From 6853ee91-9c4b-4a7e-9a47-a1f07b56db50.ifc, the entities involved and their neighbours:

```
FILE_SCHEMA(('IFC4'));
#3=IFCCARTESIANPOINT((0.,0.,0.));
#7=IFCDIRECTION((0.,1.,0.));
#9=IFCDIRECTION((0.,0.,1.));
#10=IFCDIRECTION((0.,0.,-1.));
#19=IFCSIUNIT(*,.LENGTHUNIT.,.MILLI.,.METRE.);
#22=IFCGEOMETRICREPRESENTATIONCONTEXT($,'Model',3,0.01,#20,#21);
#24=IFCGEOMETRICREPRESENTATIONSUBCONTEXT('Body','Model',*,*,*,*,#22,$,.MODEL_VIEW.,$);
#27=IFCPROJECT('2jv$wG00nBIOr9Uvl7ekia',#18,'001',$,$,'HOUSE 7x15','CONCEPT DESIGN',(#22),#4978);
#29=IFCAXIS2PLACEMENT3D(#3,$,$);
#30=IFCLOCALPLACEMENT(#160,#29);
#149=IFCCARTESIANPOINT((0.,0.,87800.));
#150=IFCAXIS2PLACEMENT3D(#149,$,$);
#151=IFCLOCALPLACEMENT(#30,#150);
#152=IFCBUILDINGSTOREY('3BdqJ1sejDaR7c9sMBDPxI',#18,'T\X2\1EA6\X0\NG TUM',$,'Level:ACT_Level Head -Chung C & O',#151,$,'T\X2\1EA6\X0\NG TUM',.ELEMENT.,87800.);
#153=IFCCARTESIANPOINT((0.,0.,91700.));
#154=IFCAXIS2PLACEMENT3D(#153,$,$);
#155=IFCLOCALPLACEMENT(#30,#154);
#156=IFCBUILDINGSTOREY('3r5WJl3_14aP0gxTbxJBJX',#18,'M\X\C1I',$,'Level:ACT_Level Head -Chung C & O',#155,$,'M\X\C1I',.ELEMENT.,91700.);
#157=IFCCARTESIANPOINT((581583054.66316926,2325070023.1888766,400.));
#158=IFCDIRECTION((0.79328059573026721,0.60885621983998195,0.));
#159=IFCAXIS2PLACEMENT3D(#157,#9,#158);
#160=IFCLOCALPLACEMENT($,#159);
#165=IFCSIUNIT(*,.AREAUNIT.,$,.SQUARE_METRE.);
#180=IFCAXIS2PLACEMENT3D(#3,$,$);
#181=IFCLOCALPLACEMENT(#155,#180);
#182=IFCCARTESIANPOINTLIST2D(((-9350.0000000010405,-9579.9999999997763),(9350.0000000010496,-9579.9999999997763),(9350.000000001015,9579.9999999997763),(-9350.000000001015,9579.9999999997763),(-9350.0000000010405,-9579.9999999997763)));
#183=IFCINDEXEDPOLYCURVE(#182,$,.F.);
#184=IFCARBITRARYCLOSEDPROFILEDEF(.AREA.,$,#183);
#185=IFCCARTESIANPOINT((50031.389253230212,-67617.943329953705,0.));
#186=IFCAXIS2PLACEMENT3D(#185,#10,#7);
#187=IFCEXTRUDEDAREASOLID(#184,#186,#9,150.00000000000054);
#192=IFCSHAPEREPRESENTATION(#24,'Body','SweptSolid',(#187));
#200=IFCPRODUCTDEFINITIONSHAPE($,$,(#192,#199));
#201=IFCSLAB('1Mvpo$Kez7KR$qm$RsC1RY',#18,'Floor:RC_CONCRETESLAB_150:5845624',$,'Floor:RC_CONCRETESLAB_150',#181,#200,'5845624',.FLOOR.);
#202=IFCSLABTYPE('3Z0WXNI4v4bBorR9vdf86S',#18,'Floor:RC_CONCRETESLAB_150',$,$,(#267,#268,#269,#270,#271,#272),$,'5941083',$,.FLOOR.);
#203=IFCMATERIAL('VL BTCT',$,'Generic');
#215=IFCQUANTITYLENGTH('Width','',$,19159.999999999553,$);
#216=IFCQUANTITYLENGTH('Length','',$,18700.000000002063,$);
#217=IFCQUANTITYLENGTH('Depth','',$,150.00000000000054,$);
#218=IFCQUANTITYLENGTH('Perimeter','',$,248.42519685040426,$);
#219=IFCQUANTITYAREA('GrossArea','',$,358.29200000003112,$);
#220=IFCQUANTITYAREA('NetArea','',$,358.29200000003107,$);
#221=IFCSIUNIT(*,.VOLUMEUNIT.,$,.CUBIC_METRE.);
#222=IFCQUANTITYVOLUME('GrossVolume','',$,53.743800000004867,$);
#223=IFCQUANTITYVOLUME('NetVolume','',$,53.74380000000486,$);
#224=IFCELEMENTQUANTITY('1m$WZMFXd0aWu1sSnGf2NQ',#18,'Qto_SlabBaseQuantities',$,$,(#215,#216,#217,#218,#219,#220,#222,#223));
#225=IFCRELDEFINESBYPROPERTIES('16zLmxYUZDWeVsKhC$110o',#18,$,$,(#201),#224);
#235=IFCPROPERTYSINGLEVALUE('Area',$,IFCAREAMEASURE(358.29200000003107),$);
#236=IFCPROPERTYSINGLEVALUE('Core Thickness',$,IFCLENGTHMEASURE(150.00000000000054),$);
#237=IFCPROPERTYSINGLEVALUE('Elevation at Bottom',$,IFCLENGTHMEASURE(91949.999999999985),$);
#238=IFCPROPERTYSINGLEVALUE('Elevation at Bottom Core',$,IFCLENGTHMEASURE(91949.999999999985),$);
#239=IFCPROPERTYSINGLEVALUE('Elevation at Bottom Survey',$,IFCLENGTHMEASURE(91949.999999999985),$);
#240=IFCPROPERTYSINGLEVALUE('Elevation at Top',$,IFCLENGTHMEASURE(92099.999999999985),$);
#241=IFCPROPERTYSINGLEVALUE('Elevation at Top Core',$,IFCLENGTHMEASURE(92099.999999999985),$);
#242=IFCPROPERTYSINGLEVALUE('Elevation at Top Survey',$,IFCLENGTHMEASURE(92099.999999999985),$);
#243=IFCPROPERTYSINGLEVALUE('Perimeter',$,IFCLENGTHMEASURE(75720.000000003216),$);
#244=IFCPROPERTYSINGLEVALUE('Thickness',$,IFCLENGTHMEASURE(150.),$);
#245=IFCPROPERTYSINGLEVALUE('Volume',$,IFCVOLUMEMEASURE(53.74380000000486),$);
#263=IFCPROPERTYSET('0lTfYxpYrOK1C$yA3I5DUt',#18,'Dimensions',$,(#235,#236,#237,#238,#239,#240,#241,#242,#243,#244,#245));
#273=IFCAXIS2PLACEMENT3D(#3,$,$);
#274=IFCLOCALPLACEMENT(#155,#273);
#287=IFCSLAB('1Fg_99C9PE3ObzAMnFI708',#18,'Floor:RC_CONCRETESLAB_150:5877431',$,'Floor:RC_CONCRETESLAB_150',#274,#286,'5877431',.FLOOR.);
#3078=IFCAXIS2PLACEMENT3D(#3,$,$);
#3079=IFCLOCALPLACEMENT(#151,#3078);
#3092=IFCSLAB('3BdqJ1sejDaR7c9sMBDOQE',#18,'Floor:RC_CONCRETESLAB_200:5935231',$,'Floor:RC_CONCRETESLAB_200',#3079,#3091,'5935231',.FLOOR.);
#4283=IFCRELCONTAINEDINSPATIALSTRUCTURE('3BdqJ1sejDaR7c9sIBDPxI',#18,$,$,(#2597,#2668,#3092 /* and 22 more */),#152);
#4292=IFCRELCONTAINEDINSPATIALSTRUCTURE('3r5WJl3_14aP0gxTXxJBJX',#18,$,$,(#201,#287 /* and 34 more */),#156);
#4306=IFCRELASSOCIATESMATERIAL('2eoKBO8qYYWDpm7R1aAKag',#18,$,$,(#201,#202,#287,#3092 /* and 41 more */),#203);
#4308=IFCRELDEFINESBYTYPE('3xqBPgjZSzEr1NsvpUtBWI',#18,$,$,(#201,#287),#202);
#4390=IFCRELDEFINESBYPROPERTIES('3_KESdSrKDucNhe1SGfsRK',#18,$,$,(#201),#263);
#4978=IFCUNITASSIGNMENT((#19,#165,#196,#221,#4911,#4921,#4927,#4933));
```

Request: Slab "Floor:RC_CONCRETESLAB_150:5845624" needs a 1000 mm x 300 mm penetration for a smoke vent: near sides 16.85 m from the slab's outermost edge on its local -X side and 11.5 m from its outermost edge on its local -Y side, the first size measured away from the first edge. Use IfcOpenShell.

```python
import numpy as np
import ifcopenshell
import ifcopenshell.api.feature
import ifcopenshell.api.geometry
import ifcopenshell.api.pset
import ifcopenshell.api.root
import ifcopenshell.geom
import ifcopenshell.util.element
import ifcopenshell.util.placement
import ifcopenshell.util.representation
import ifcopenshell.util.shape
import ifcopenshell.util.unit

model = ifcopenshell.open("6853ee91-9c4b-4a7e-9a47-a1f07b56db50.ifc")
unit_scale = ifcopenshell.util.unit.calculate_unit_scale(model)
area_scale = ifcopenshell.util.unit.calculate_unit_scale(model, "AREAUNIT")
volume_scale = ifcopenshell.util.unit.calculate_unit_scale(model, "VOLUMEUNIT")
settings = ifcopenshell.geom.settings()


def volume(element):
    """Net volume in cubic metres, openings subtracted."""
    shape = ifcopenshell.geom.create_shape(settings, element)
    return ifcopenshell.util.shape.get_volume(shape.geometry)


slab = model.by_guid("1Mvpo$Kez7KR$qm$RsC1RY")
before = volume(slab)

# Extent in the slab's own axes, in metres. The edges named are its -X and -Y sides.
slab_shape = ifcopenshell.geom.create_shape(settings, slab)
vertices = ifcopenshell.util.shape.get_vertices(slab_shape.geometry)
x_min, y_min, bottom = vertices.min(axis=0)
top = vertices[:, 2].max()

opening = ifcopenshell.api.root.create_entity(model, ifc_class="IfcOpeningElement", name="Smoke vent opening", predefined_type="OPENING")
context = ifcopenshell.util.representation.get_context(model, "Model", "Body", "MODEL_VIEW")
width, depth = 1, 0.3
outline = [(0.0, 0.0), (width, 0.0), (width, depth), (0.0, depth), (0.0, 0.0)]
# Overshoot both faces by 50 mm so the cut is clean.
shape = ifcopenshell.api.geometry.add_slab_representation(
    model, context=context, depth=top - bottom + 0.1, polyline=outline
)
ifcopenshell.api.geometry.assign_representation(model, product=opening, representation=shape)

matrix = ifcopenshell.util.placement.get_local_placement(slab.ObjectPlacement)
matrix[:, 3] = matrix @ np.append(np.array([x_min + 16.85, y_min + 11.5, bottom - 0.05]) / unit_scale, 1.0)
ifcopenshell.api.geometry.edit_object_placement(model, product=opening, matrix=matrix, is_si=False)
ifcopenshell.api.feature.add_feature(model, feature=opening, element=slab)

after = volume(slab)

# Update the slab's stored quantities.
qto = model.by_id(ifcopenshell.util.element.get_pset(slab, "Qto_SlabBaseQuantities", should_inherit=False)["id"])
ifcopenshell.api.pset.edit_qto(model, qto=qto, properties={
    "NetArea": after / (top - bottom) / area_scale,
    "NetVolume": after / volume_scale,
})
pset = model.by_id(ifcopenshell.util.element.get_pset(slab, "Dimensions", should_inherit=False)["id"])
ifcopenshell.api.pset.edit_pset(model, pset=pset, properties={
    "Area": model.create_entity("IfcAreaMeasure", after / (top - bottom) / area_scale),
    "Volume": model.create_entity("IfcVolumeMeasure", after / volume_scale),
})

print(f"slab volume {before:.3f} -> {after:.3f} m3")

model.write("6853ee91-9c4b-4a7e-9a47-a1f07b56db50-out.ifc")
```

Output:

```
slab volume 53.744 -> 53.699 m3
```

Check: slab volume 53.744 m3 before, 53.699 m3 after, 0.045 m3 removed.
